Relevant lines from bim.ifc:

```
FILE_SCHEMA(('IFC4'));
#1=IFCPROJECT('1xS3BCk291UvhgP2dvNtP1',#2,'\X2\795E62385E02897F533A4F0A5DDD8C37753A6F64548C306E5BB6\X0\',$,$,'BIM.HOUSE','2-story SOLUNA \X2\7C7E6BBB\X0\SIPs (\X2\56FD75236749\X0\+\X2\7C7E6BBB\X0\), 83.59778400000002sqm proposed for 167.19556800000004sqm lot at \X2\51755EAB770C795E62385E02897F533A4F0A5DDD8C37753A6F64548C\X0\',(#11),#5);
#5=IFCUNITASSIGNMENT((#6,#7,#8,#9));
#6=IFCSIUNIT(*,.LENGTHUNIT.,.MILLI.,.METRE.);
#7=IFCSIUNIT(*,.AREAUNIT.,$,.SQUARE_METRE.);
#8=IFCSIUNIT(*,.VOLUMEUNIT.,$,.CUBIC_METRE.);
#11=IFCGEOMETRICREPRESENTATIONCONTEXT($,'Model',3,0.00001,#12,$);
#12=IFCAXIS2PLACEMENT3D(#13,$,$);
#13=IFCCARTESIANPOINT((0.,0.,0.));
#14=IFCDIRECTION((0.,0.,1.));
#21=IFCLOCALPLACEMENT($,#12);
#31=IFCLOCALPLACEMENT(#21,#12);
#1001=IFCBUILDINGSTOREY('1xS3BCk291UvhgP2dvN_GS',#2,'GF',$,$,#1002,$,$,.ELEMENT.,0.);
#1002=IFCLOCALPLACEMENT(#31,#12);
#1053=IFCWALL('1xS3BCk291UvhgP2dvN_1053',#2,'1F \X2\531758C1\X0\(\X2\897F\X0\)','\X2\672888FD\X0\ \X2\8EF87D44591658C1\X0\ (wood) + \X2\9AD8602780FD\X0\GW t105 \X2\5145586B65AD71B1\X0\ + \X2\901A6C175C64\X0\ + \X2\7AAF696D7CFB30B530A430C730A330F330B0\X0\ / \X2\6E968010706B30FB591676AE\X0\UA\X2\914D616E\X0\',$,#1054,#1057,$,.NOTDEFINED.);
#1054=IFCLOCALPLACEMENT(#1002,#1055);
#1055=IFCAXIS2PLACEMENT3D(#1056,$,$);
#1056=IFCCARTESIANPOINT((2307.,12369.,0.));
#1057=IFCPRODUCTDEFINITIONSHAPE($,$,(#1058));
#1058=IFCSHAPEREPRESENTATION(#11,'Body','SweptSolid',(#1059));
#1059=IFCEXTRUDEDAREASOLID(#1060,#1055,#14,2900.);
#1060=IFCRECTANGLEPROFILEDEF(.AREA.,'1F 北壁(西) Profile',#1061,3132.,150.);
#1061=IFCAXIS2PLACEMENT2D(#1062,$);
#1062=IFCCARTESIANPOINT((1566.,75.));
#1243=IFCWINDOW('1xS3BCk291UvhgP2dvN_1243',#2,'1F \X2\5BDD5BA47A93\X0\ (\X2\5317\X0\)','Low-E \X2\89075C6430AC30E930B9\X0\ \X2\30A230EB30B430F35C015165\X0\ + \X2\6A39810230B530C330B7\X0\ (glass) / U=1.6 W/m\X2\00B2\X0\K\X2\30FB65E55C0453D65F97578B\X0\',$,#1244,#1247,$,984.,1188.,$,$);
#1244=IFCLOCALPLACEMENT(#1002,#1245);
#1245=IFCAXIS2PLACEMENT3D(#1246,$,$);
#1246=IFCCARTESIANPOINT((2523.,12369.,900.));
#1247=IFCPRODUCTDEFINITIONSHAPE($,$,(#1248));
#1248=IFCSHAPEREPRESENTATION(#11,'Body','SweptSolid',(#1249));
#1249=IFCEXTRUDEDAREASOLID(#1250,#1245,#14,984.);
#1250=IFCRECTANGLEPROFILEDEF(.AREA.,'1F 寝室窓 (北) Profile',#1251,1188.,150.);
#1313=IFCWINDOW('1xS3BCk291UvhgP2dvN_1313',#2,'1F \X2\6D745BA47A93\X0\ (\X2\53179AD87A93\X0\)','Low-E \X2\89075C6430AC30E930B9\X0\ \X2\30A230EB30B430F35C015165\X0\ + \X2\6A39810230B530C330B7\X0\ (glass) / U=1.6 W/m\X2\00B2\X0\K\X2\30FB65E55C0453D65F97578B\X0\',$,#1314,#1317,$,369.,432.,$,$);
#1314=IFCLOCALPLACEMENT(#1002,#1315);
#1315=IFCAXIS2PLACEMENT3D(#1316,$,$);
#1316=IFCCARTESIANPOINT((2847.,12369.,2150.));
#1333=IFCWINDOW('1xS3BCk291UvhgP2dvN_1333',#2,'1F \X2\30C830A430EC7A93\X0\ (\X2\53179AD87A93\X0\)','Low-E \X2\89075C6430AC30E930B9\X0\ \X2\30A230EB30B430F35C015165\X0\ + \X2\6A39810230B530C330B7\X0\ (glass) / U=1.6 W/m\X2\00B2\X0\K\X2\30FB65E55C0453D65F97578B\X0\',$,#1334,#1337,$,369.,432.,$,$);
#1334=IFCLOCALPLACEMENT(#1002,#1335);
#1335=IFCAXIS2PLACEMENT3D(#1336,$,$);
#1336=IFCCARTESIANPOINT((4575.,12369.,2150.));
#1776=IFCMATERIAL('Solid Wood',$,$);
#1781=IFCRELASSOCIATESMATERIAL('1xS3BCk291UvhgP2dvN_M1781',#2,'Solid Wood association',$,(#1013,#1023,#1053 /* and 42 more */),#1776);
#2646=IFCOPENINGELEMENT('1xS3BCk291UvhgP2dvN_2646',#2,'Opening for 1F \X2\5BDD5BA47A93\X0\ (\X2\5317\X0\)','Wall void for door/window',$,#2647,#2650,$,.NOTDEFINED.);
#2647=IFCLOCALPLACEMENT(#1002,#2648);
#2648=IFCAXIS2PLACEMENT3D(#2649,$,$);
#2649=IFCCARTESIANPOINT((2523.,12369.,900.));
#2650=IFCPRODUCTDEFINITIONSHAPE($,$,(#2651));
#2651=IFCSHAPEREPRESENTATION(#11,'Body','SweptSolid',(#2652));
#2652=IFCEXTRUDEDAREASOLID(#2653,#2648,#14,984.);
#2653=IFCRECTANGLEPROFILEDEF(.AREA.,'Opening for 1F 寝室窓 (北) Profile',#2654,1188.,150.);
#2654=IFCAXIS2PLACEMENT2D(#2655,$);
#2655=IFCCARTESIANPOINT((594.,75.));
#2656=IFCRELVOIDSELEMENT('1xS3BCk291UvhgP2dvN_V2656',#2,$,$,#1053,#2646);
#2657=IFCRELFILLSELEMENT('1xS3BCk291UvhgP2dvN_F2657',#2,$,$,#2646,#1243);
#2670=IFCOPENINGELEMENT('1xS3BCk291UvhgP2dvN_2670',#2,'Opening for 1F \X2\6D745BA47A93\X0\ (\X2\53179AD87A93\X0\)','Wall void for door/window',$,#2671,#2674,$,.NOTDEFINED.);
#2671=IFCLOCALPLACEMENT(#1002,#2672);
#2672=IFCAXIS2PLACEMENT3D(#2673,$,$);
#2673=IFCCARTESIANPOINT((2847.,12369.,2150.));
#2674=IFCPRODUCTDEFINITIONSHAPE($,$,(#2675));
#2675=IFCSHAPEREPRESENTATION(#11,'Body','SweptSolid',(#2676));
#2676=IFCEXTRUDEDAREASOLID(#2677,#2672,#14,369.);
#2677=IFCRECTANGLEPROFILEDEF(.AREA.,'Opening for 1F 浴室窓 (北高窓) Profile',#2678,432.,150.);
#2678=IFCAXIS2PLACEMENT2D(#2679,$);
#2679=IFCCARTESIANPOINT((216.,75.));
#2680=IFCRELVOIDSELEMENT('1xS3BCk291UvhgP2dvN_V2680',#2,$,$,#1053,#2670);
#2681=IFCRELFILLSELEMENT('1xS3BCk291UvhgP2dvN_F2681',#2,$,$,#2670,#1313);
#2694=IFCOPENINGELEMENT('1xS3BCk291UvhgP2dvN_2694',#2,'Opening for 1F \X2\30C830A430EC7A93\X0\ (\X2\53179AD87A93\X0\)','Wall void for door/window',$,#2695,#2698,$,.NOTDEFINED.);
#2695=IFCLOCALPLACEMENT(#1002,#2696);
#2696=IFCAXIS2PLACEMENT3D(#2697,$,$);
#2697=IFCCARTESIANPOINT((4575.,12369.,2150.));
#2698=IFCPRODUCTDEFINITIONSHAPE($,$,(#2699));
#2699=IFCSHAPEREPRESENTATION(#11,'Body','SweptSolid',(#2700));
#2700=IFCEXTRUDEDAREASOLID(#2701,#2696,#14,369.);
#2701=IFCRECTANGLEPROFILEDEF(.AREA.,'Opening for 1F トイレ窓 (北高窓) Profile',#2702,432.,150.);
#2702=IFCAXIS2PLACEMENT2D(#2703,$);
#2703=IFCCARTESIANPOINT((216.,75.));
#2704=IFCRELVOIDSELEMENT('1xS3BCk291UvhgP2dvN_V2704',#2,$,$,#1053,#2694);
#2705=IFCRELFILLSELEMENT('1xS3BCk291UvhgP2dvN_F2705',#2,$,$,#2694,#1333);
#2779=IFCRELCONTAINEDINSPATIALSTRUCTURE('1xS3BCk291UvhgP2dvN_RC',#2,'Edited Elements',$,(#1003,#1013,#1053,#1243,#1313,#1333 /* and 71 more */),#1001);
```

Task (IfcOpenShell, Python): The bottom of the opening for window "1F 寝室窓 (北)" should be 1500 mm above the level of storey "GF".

```python
import numpy as np
import ifcopenshell
import ifcopenshell.api.geometry
import ifcopenshell.geom
import ifcopenshell.util.element
import ifcopenshell.util.placement
import ifcopenshell.util.shape
import ifcopenshell.util.unit

model = ifcopenshell.open("bim.ifc")
unit_scale = ifcopenshell.util.unit.calculate_unit_scale(model)

window = model.by_guid("1xS3BCk291UvhgP2dvN_1243")
opening = window.FillsVoids[0].RelatingOpeningElement
storey = ifcopenshell.util.element.get_container(window, ifc_class="IfcBuildingStorey")
level = ifcopenshell.util.placement.get_local_placement(storey.ObjectPlacement)[2, 3]

# The opening's origin need not be at the sill, so measure its lowest point.
shape = ifcopenshell.geom.create_shape(ifcopenshell.geom.settings(), opening)
bottom = ifcopenshell.util.shape.get_shape_bottom_elevation(shape, shape.geometry) / unit_scale
dz = level + 1.5 / unit_scale - bottom

shift = np.array([0.0, 0.0, dz])
# The window is not placed relative to its opening, so move both.
for product in (opening, window):
    matrix = ifcopenshell.util.placement.get_local_placement(product.ObjectPlacement)
    matrix[:3, 3] += shift
    ifcopenshell.api.geometry.edit_object_placement(model, product=product, matrix=matrix, is_si=False)

print(f"moved by {dz * unit_scale:+.3f} m")

model.write("bim_edited.ifc")
```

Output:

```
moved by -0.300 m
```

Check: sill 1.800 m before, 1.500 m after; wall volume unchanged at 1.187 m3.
